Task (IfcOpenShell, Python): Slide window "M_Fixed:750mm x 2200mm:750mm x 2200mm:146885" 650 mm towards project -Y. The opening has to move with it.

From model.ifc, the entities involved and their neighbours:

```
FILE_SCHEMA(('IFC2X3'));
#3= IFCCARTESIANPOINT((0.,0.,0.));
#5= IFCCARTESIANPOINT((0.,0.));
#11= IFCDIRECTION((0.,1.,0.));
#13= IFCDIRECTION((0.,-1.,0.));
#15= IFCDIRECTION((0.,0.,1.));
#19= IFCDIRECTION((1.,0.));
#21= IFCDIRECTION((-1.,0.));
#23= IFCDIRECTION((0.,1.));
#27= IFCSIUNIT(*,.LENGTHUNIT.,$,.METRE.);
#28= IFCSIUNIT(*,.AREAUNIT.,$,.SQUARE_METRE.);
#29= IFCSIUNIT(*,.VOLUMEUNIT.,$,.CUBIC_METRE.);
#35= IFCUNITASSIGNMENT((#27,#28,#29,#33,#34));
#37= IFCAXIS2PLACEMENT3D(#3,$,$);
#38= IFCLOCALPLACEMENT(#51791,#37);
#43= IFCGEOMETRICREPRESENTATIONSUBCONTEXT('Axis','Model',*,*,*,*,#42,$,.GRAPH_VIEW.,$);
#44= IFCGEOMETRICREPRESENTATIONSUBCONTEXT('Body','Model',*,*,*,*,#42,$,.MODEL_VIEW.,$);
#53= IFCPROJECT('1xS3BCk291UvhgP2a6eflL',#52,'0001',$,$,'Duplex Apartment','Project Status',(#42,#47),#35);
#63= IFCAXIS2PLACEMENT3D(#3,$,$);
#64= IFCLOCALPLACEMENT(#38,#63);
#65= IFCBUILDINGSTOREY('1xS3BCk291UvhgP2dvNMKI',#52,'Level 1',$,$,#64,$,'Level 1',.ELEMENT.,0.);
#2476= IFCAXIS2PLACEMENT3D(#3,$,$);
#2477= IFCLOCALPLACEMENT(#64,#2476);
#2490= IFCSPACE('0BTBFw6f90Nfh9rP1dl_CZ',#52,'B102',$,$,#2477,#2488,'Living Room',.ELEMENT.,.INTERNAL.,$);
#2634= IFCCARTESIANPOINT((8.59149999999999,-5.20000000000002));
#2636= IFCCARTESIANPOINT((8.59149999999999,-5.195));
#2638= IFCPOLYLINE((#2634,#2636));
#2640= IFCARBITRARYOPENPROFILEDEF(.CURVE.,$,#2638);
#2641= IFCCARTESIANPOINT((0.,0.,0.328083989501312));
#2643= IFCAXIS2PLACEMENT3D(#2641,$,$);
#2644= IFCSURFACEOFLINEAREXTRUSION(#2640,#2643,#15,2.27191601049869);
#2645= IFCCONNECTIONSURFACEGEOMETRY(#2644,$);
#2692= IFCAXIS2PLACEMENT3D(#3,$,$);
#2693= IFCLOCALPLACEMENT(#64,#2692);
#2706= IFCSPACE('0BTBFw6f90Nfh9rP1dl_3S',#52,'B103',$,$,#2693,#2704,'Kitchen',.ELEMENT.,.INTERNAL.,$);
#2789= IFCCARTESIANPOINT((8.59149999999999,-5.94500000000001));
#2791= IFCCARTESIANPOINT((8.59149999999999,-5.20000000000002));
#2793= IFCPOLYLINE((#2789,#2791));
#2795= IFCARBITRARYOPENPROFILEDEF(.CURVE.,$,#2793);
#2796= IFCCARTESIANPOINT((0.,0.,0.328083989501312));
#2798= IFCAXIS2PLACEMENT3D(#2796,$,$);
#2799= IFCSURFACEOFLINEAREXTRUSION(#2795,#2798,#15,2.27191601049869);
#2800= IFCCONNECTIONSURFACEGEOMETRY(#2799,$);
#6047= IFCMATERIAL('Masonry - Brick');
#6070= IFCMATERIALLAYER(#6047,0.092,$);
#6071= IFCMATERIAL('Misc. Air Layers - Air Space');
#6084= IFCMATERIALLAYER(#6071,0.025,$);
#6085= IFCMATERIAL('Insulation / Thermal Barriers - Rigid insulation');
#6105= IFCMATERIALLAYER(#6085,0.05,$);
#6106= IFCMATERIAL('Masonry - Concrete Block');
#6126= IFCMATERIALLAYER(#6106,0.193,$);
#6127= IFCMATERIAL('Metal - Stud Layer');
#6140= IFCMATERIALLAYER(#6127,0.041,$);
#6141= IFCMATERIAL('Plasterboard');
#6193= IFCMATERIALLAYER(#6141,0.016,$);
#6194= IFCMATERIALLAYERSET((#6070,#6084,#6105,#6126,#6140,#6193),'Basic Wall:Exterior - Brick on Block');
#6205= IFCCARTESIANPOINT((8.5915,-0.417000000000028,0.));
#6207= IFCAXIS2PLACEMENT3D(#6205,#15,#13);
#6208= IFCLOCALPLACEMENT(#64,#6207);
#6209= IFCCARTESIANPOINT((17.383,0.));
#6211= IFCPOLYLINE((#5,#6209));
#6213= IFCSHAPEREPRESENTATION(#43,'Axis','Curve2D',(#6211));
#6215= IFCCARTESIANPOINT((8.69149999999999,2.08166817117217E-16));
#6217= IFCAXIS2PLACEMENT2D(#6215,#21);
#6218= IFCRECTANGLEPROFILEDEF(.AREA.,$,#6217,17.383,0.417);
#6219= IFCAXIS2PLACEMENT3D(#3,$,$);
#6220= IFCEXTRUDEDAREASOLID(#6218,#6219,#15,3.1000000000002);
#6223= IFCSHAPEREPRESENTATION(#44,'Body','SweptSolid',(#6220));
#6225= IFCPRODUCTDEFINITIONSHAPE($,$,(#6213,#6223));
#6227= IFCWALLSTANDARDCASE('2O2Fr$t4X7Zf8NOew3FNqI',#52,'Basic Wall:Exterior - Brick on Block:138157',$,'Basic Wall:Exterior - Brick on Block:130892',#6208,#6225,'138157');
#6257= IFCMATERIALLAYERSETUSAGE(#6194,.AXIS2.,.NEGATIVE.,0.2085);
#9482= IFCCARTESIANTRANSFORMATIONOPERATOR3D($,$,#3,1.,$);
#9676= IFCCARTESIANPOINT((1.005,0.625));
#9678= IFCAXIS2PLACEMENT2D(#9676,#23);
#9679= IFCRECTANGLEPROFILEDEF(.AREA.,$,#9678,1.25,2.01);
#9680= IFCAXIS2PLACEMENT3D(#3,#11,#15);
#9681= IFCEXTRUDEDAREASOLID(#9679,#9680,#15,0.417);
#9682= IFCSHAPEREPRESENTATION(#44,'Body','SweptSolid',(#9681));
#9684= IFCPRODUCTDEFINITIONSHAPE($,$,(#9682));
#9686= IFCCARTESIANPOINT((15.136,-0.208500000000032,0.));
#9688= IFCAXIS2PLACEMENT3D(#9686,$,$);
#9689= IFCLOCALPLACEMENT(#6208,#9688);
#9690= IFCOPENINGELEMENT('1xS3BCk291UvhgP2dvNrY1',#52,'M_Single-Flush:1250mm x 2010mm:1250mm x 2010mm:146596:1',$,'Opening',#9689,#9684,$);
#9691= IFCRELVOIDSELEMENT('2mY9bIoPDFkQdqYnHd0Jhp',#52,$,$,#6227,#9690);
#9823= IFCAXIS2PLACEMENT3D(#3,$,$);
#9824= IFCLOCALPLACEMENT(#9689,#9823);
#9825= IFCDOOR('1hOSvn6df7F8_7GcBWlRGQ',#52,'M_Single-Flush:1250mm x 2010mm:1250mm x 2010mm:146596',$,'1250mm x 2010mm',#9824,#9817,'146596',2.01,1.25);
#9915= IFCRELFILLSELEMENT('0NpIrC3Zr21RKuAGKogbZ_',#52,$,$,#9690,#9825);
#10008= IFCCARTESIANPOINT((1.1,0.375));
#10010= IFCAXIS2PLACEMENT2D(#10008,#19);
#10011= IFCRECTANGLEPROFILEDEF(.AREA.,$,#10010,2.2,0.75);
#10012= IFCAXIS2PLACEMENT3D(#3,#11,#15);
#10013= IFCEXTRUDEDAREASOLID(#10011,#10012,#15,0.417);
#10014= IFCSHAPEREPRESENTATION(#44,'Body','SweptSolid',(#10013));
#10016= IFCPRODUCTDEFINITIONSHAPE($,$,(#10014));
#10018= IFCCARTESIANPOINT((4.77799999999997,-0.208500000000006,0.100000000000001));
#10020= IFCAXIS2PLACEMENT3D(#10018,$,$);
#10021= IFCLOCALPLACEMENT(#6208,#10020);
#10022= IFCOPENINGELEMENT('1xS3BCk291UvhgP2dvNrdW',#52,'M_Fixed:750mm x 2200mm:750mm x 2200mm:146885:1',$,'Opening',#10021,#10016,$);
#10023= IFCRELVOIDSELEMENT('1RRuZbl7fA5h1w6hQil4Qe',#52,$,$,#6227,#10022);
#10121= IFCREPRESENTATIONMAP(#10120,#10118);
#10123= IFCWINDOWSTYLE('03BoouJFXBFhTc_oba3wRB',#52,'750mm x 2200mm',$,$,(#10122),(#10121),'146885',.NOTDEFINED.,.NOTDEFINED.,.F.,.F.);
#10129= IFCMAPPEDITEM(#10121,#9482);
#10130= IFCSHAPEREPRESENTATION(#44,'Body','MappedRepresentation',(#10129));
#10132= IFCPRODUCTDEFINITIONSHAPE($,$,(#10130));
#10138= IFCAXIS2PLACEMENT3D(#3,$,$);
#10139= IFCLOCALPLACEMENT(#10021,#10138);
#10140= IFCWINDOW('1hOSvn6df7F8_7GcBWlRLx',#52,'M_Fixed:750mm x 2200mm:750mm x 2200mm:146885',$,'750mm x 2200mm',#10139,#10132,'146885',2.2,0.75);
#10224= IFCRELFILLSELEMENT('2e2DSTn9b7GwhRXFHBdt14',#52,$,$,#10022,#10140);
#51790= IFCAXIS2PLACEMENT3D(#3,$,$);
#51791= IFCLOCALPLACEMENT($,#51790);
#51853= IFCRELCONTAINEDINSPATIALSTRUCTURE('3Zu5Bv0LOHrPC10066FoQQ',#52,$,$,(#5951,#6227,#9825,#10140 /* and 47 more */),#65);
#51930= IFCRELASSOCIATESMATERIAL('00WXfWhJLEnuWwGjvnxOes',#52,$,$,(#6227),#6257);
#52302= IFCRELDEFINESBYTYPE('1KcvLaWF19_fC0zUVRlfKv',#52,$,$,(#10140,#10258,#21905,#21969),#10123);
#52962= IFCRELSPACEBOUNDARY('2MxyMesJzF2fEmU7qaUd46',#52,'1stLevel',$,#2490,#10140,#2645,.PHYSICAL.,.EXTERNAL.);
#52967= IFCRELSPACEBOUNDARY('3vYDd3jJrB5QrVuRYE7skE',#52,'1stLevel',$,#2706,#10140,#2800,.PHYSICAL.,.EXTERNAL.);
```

```python
import numpy as np
import ifcopenshell
import ifcopenshell.api.geometry
import ifcopenshell.util.placement
import ifcopenshell.util.unit

model = ifcopenshell.open("model.ifc")
unit_scale = ifcopenshell.util.unit.calculate_unit_scale(model)

window = model.by_guid("1hOSvn6df7F8_7GcBWlRLx")
opening = window.FillsVoids[0].RelatingOpeningElement
wall = opening.VoidsElements[0].RelatingBuildingElement

wall_matrix = ifcopenshell.util.placement.get_local_placement(wall.ObjectPlacement)
shift = wall_matrix[:3, 0] * 0.65 / unit_scale
before = ifcopenshell.util.placement.get_local_placement(window.ObjectPlacement)[:3, 3].copy()

# The window is placed relative to its opening, so it follows when the opening moves.
matrix = ifcopenshell.util.placement.get_local_placement(opening.ObjectPlacement)
matrix[:3, 3] += shift
ifcopenshell.api.geometry.edit_object_placement(
    model, product=opening, matrix=matrix, is_si=False, should_transform_children=True
)

# Space boundary surfaces are stored in each space's coordinates; move them too.
for rel in window.ProvidesBoundaries:
    if not rel.ConnectionGeometry:
        continue
    surface = rel.ConnectionGeometry.SurfaceOnRelatingElement
    space_matrix = ifcopenshell.util.placement.get_local_placement(rel.RelatingSpace.ObjectPlacement)
    point = np.array(surface.Position.Location.Coordinates) + space_matrix[:3, :3].T @ shift
    surface.Position = model.createIfcAxis2Placement3D(
        model.createIfcCartesianPoint(point.tolist()), surface.Position.Axis, surface.Position.RefDirection
    )

after = ifcopenshell.util.placement.get_local_placement(window.ObjectPlacement)[:3, 3]
print("window moved by", (after - before).round(3) + 0.0)

model.write("model_v2.ifc")
```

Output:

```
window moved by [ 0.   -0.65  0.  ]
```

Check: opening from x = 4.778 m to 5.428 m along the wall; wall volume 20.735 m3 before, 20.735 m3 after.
